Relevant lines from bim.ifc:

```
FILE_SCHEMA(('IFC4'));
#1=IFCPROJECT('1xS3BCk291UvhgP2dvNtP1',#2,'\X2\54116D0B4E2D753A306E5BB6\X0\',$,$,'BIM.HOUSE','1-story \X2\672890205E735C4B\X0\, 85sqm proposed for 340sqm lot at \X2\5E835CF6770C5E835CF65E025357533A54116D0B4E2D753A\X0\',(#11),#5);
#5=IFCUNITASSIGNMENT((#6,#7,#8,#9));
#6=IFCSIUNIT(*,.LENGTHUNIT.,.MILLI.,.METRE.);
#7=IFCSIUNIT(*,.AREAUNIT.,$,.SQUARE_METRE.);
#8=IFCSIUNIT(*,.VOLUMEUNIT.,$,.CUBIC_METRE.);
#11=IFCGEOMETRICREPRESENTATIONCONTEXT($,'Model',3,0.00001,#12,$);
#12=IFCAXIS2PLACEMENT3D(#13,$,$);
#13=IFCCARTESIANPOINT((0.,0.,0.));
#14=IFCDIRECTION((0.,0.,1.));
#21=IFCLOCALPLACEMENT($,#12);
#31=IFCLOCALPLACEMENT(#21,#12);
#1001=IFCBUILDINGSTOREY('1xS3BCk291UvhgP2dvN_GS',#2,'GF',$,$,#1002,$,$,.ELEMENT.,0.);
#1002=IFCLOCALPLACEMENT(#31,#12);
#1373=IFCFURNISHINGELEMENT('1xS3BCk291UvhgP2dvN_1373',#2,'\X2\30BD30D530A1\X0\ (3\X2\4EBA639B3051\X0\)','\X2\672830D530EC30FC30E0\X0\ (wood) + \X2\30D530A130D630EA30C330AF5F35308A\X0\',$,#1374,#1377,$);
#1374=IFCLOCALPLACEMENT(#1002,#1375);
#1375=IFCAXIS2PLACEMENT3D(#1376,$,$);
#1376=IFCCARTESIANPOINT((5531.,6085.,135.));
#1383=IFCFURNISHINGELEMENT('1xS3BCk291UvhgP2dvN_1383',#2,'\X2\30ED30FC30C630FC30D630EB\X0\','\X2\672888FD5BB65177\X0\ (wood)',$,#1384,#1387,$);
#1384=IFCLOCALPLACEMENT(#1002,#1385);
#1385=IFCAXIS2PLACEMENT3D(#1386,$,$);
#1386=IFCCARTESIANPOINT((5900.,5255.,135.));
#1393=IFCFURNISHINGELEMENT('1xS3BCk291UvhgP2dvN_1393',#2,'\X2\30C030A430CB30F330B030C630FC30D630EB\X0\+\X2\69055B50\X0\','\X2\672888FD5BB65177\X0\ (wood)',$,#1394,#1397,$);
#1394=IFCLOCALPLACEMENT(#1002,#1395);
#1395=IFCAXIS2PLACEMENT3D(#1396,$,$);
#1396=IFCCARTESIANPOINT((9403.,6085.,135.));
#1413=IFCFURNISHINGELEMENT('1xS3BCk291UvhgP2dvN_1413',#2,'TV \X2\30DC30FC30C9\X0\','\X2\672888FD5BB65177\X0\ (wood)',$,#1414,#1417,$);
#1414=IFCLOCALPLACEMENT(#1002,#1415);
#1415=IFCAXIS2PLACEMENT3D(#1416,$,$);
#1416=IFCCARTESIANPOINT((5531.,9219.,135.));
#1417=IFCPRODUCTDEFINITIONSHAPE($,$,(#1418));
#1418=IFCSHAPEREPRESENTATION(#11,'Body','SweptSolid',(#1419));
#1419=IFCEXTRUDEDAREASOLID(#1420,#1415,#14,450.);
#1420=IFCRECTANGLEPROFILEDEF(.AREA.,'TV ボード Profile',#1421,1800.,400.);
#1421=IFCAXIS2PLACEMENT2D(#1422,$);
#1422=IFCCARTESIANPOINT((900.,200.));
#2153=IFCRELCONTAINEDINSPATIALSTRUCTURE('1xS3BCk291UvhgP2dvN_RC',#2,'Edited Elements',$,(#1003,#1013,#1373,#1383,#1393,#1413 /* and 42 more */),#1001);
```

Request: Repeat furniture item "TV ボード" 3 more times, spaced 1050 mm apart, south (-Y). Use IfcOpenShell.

```python
import numpy as np
import ifcopenshell
import ifcopenshell.api.geometry
import ifcopenshell.api.root
import ifcopenshell.util.element
import ifcopenshell.util.placement
import ifcopenshell.util.unit

model = ifcopenshell.open("bim.ifc")
unit_scale = ifcopenshell.util.unit.calculate_unit_scale(model)


def reuse_history(source, copy):
    """copy_class also copies each property set's owner history, people and application; keep the originals."""
    for rel in copy.IsDefinedBy:
        if rel.is_a("IfcRelDefinesByProperties") and (history := rel.RelatingPropertyDefinition.OwnerHistory):
            rel.RelatingPropertyDefinition.OwnerHistory = source.OwnerHistory
            ifcopenshell.util.element.remove_deep2(model, history)


source = model.by_guid("1xS3BCk291UvhgP2dvN_1413")
base = ifcopenshell.util.placement.get_local_placement(source.ObjectPlacement)
step = np.array([0.0, -1.0, 0.0]) * 1.05 / unit_scale

for i in range(1, 4):
    copy = ifcopenshell.api.root.copy_class(model, product=source)
    copy.Representation = ifcopenshell.util.element.copy_deep(
        model, source.Representation, exclude=["IfcGeometricRepresentationContext", "IfcRepresentationMap"]
    )
    reuse_history(source, copy)
    matrix = base.copy()
    matrix[:3, 3] += i * step
    print("added at", matrix[:3, 3].round(3) + 0.0)
    ifcopenshell.api.geometry.edit_object_placement(model, product=copy, matrix=matrix, is_si=False)

model.write("bim_updated.ifc")
```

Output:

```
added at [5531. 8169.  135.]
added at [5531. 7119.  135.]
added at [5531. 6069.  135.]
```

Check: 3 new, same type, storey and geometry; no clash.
